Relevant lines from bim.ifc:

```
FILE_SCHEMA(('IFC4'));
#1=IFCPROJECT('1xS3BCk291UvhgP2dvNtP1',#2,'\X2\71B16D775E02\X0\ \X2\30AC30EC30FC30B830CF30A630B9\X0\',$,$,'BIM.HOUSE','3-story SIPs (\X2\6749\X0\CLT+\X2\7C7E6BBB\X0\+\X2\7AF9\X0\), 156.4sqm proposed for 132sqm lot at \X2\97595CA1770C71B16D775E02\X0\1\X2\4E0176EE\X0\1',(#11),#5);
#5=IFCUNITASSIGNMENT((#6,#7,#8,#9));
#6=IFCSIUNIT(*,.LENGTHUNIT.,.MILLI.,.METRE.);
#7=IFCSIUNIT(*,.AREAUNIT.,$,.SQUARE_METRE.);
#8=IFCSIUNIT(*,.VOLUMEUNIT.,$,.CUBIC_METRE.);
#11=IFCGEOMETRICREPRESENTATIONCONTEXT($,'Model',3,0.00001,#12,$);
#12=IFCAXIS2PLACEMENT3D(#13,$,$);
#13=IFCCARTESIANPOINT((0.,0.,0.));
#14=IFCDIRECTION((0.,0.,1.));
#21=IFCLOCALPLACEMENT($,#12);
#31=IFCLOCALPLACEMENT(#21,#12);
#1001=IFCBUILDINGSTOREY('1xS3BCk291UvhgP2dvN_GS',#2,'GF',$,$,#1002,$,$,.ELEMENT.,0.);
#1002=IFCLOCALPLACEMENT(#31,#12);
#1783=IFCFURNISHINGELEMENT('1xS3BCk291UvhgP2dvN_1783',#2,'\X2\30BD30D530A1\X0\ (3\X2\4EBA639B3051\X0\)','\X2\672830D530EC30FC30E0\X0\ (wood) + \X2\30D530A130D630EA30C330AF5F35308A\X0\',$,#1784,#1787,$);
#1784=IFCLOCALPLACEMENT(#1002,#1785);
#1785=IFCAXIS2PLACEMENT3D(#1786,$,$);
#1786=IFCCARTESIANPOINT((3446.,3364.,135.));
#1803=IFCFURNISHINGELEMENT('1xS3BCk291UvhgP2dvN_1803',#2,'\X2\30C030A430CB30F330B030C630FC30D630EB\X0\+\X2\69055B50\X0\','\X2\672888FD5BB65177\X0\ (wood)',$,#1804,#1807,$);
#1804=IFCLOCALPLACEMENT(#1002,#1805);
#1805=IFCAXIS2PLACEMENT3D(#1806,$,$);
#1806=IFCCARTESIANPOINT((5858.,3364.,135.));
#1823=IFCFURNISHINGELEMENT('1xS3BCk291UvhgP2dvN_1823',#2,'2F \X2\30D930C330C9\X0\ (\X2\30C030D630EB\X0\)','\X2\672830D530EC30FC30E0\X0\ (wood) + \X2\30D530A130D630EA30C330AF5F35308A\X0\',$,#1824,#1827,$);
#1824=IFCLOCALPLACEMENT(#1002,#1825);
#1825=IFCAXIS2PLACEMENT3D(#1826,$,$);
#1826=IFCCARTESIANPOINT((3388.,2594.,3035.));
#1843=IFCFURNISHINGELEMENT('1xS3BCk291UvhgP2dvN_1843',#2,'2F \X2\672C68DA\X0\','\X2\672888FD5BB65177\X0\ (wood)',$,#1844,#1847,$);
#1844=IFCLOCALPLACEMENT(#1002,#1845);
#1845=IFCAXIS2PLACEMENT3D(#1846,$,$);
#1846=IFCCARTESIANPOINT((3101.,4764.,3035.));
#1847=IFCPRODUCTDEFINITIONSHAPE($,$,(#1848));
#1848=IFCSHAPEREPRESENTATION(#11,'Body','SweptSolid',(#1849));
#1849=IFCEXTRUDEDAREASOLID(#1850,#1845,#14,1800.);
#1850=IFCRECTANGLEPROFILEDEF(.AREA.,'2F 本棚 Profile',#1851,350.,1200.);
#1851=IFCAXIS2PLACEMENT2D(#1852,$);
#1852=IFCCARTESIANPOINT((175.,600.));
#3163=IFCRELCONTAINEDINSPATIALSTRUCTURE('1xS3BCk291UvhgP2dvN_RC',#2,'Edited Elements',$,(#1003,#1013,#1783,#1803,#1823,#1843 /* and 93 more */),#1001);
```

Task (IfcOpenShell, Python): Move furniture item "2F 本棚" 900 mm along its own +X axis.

```python
import ifcopenshell
import ifcopenshell.api.geometry
import ifcopenshell.util.placement
import ifcopenshell.util.unit

model = ifcopenshell.open("bim.ifc")
unit_scale = ifcopenshell.util.unit.calculate_unit_scale(model)

item = model.by_guid("1xS3BCk291UvhgP2dvN_1843")
matrix = ifcopenshell.util.placement.get_local_placement(item.ObjectPlacement)
matrix[:3, 3] += matrix[:3, 0] * 0.9 / unit_scale
ifcopenshell.api.geometry.edit_object_placement(model, product=item, matrix=matrix, is_si=False)

print(ifcopenshell.util.placement.get_local_placement(item.ObjectPlacement).round(3) + 0.0)

model.write("bim_rev.ifc")
```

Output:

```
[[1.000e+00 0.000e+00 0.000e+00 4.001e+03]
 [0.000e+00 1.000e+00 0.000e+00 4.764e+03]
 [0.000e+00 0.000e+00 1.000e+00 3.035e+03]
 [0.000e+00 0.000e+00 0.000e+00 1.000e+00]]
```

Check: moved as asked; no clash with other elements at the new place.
